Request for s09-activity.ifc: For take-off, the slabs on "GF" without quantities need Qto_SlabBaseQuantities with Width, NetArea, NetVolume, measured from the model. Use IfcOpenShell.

First a look at what the model holds.

```python
import ifcopenshell
import ifcopenshell.util.element
import ifcopenshell.util.unit

model = ifcopenshell.open("s09-activity.ifc")
print(model.schema)
for unit_type in ("LENGTHUNIT", "AREAUNIT", "VOLUMEUNIT"):
    print(unit_type, ifcopenshell.util.unit.calculate_unit_scale(model, unit_type))
storey = next(s for s in model.by_type("IfcBuildingStorey") if s.Name == "GF")
slabs = [e for e in ifcopenshell.util.element.get_decomposition(storey) if e.is_a("IfcSlab")]
for e in sorted(slabs, key=lambda e: e.id()):
    print(e.id(), e.is_a(), e.Name, list(ifcopenshell.util.element.get_psets(e, qtos_only=True)), sep=" | ")
```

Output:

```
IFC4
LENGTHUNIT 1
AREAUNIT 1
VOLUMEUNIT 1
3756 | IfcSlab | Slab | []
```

```python
import ifcopenshell
import ifcopenshell.api.pset
import ifcopenshell.geom
import ifcopenshell.util.element
import ifcopenshell.util.shape
import ifcopenshell.util.unit

model = ifcopenshell.open("s09-activity.ifc")
unit_scale = ifcopenshell.util.unit.calculate_unit_scale(model)
area_scale = ifcopenshell.util.unit.calculate_unit_scale(model, "AREAUNIT")
volume_scale = ifcopenshell.util.unit.calculate_unit_scale(model, "VOLUMEUNIT")
settings = ifcopenshell.geom.settings()

storey = next(s for s in model.by_type("IfcBuildingStorey") if s.Name == "GF")
slabs = [e for e in ifcopenshell.util.element.get_decomposition(storey) if e.is_a("IfcSlab")]

for e in sorted(slabs, key=lambda e: e.id()):
    if ifcopenshell.util.element.get_psets(e, qtos_only=True, should_inherit=False):
        continue
    # Geometry comes back in metres, in the element's own axes.
    shape = ifcopenshell.geom.create_shape(settings, e)
    values = {
        "Width": ifcopenshell.util.shape.get_z(shape.geometry) / unit_scale,
        "NetArea": ifcopenshell.util.shape.get_footprint_area(shape.geometry) / area_scale,
        "NetVolume": ifcopenshell.util.shape.get_volume(shape.geometry) / volume_scale,
    }
    qto = ifcopenshell.api.pset.add_qto(model, product=e, name="Qto_SlabBaseQuantities")
    ifcopenshell.api.pset.edit_qto(model, qto=qto, properties=values)
    print(e.id(), {k: round(v, 3) for k, v in values.items()})

model.write("s09-activity_rev.ifc")
```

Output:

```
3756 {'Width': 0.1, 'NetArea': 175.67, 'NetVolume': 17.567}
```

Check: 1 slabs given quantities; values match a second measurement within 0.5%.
